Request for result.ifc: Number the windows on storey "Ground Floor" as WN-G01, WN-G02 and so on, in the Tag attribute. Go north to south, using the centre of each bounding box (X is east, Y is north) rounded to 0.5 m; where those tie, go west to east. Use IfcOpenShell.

First a look at what the model holds.

```python
import ifcopenshell
import ifcopenshell.util.element
import ifcopenshell.util.placement

model = ifcopenshell.open("result.ifc")
print(model.schema)
storey = next(s for s in model.by_type("IfcBuildingStorey") if s.Name == "Ground Floor")
windows = [e for e in ifcopenshell.util.element.get_decomposition(storey) if e.is_a("IfcWindow")]
for e in sorted(windows, key=lambda e: e.id()):
    origin = ifcopenshell.util.placement.get_local_placement(e.ObjectPlacement)[:3, 3]
    print(e.id(), e.Tag, e.Name, origin.round(2) + 0.0, sep=" | ")
```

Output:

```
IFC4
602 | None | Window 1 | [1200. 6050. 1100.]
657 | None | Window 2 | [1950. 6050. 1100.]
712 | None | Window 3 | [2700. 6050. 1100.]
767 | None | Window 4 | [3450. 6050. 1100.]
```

```python
import ifcopenshell
import ifcopenshell.geom
import ifcopenshell.util.element
import ifcopenshell.util.shape

model = ifcopenshell.open("result.ifc")
settings = ifcopenshell.geom.settings()
settings.set("use-world-coords", True)


def centre(element):
    shape = ifcopenshell.geom.create_shape(settings, element)
    return ifcopenshell.util.shape.get_bbox_centroid(shape.geometry)


storey = next(s for s in model.by_type("IfcBuildingStorey") if s.Name == "Ground Floor")
windows = [e for e in ifcopenshell.util.element.get_decomposition(storey) if e.is_a("IfcWindow")]

# Insertion points can sit at a corner or the storey origin, so sort by the geometry (in metres).
centres = {e: centre(e) for e in windows}
windows.sort(key=lambda e: (-round(centres[e][1] / 0.5), centres[e][0]))

for i, e in enumerate(windows, start=1):
    number = f"WN-G{i:02d}"
    e.Tag = number
    print(e.id(), number)

model.write("result_v2.ifc")
```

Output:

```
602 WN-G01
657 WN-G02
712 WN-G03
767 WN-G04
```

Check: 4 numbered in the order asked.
